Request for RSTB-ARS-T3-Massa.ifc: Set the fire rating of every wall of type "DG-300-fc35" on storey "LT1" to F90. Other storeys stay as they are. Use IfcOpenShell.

First a look at what the model holds.

```python
import ifcopenshell
import ifcopenshell.util.element

model = ifcopenshell.open("RSTB-ARS-T3-Massa.ifc")
print(model.schema)
storey = next(s for s in model.by_type("IfcBuildingStorey") if s.Name == "LT1")
walls = [e for e in ifcopenshell.util.element.get_decomposition(storey) if e.is_a("IfcWall")]
seen = {}
for e in walls:
    element_type = ifcopenshell.util.element.get_type(e)
    key = (element_type.Name if element_type != e and element_type else None, ifcopenshell.util.element.get_pset(e, "Pset_WallCommon", "FireRating"))
    seen[key] = seen.get(key, 0) + 1
for (name, value), count in sorted(seen.items(), key=str):
    print(count, "x", name, "|", value)
```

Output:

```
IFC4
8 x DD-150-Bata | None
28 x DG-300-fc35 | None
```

```python
import ifcopenshell
import ifcopenshell.api.pset
import ifcopenshell.util.element

model = ifcopenshell.open("RSTB-ARS-T3-Massa.ifc")

storey = next(s for s in model.by_type("IfcBuildingStorey") if s.Name == "LT1")
walls = [e for e in ifcopenshell.util.element.get_decomposition(storey) if e.is_a("IfcWall")]

count = 0
for e in walls:
    element_type = ifcopenshell.util.element.get_type(e)
    if element_type in (None, e) or element_type.Name != "DG-300-fc35":
        continue
    # add_pset returns the element's existing set when there is one.
    pset = ifcopenshell.api.pset.add_pset(model, product=e, name="Pset_WallCommon")
    ifcopenshell.api.pset.edit_pset(model, pset=pset, properties={"FireRating": "F90"})
    count += 1

print(count, "walls updated")

model.write("RSTB-ARS-T3-Massa_rev.ifc")
```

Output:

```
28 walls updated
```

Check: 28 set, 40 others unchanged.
